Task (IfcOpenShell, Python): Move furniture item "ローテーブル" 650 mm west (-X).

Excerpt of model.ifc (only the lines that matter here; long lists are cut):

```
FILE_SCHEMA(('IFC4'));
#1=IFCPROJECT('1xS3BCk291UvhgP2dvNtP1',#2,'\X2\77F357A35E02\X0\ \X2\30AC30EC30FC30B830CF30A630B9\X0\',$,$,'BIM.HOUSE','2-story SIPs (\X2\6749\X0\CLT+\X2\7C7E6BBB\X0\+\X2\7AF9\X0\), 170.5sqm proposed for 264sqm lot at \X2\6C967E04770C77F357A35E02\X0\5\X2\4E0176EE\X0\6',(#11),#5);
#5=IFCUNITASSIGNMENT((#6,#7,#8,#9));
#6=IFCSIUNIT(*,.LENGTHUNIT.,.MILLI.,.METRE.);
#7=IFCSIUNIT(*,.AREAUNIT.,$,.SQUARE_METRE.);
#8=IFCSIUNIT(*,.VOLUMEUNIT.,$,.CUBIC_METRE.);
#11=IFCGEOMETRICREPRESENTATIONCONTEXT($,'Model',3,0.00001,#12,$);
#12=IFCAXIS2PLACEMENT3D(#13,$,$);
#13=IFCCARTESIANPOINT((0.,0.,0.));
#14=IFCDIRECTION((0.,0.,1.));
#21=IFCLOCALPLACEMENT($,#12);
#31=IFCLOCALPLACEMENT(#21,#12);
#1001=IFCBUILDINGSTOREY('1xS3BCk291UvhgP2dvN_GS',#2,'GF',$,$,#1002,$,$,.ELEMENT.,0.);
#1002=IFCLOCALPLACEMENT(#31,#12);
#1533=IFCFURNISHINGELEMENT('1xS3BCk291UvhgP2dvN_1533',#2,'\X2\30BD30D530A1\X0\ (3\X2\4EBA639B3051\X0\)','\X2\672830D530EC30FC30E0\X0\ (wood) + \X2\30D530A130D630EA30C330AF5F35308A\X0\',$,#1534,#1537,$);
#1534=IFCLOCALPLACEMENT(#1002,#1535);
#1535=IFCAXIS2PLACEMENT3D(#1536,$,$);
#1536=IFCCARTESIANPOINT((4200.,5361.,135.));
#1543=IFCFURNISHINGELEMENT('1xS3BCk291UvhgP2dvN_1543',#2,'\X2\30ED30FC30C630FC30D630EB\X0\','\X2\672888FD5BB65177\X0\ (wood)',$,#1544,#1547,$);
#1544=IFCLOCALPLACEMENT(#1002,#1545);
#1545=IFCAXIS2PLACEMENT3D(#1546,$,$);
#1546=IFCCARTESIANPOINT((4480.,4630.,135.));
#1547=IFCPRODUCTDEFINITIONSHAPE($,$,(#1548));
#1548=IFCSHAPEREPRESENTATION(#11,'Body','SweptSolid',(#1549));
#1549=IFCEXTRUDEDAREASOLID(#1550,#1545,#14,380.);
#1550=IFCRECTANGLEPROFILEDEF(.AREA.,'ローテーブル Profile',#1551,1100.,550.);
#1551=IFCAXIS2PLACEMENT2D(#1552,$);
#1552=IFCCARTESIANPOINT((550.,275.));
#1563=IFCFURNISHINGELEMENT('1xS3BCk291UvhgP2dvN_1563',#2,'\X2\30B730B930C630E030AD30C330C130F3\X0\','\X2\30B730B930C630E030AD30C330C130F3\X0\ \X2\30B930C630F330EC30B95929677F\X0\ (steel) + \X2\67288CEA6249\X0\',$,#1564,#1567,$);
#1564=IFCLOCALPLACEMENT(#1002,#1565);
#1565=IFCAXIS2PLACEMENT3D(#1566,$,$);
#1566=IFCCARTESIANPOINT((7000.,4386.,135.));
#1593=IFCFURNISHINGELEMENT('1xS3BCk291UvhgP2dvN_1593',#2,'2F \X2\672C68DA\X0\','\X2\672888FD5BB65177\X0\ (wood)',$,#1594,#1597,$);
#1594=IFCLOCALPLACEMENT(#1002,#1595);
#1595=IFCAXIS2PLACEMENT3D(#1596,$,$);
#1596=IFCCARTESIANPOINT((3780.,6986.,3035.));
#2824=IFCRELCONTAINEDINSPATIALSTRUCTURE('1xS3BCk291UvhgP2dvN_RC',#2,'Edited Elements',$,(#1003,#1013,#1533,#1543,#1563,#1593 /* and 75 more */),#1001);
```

```python
import ifcopenshell
import ifcopenshell.api.geometry
import ifcopenshell.util.placement

model = ifcopenshell.open("model.ifc")

item = model.by_guid("1xS3BCk291UvhgP2dvN_1543")
matrix = ifcopenshell.util.placement.get_local_placement(item.ObjectPlacement)
matrix[0, 3] -= 650.0
ifcopenshell.api.geometry.edit_object_placement(model, product=item, matrix=matrix, is_si=False)

print(ifcopenshell.util.placement.get_local_placement(item.ObjectPlacement).round(3) + 0.0)

model.write("model_rev.ifc")
```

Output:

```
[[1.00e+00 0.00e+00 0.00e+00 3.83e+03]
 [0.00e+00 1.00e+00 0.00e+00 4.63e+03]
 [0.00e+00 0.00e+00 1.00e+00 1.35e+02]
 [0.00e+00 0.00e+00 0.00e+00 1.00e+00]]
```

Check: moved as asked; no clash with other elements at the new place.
